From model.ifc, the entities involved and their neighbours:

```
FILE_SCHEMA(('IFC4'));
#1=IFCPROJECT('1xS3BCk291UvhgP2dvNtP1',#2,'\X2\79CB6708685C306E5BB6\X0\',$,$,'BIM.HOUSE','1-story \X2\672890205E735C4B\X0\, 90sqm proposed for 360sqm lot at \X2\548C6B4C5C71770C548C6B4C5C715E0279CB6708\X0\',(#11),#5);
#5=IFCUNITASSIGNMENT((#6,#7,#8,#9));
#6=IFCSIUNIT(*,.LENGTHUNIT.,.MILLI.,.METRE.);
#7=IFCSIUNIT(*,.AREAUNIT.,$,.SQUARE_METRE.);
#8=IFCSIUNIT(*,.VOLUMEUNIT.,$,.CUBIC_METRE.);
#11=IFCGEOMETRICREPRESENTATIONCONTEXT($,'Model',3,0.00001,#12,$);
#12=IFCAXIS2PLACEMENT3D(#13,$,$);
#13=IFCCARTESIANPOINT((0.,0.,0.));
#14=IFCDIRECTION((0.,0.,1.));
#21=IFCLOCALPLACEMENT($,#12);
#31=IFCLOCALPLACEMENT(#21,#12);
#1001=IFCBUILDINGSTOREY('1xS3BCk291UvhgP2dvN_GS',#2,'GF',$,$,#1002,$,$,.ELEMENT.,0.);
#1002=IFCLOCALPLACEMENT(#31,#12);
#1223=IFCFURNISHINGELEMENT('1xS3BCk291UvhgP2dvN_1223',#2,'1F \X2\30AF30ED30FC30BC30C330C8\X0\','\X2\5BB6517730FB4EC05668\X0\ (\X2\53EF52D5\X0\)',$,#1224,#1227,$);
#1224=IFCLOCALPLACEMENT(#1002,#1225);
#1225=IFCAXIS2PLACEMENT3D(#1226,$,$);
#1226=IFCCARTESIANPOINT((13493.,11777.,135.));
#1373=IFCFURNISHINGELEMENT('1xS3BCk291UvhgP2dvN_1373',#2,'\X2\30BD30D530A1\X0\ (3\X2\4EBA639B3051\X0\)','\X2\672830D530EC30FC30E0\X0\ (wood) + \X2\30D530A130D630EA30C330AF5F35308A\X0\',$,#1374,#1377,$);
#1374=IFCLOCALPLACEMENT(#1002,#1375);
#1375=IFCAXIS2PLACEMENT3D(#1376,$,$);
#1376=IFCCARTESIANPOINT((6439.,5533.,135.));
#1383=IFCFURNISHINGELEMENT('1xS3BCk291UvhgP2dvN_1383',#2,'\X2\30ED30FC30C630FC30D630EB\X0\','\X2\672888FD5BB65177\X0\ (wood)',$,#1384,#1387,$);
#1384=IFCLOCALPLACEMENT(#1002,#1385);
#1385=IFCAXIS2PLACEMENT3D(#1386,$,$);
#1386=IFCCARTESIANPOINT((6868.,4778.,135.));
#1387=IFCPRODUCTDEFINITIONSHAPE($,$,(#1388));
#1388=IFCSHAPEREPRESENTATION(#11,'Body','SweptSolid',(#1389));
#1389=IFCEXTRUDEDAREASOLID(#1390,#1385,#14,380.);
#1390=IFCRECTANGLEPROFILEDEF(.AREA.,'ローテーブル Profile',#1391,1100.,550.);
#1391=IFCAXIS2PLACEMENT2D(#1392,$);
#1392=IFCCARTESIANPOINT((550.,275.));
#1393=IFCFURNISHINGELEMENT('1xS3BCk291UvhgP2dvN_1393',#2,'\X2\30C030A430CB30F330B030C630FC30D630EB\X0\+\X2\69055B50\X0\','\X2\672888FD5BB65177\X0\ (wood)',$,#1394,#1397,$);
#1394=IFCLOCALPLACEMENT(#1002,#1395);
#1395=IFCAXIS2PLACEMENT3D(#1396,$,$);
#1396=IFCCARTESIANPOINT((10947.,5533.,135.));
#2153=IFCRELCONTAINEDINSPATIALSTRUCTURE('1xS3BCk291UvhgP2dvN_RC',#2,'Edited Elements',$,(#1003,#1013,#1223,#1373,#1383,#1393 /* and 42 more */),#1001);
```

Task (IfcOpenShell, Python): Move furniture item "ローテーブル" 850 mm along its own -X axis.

```python
import ifcopenshell
import ifcopenshell.api.geometry
import ifcopenshell.util.placement
import ifcopenshell.util.unit

model = ifcopenshell.open("model.ifc")
unit_scale = ifcopenshell.util.unit.calculate_unit_scale(model)

item = model.by_guid("1xS3BCk291UvhgP2dvN_1383")
matrix = ifcopenshell.util.placement.get_local_placement(item.ObjectPlacement)
matrix[:3, 3] -= matrix[:3, 0] * 0.85 / unit_scale
ifcopenshell.api.geometry.edit_object_placement(model, product=item, matrix=matrix, is_si=False)

print(ifcopenshell.util.placement.get_local_placement(item.ObjectPlacement).round(3) + 0.0)

model.write("model_updated.ifc")
```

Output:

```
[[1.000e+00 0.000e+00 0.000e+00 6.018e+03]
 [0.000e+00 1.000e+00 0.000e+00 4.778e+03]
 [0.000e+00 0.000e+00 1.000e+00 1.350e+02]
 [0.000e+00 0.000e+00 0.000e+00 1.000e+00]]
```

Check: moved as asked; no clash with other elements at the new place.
